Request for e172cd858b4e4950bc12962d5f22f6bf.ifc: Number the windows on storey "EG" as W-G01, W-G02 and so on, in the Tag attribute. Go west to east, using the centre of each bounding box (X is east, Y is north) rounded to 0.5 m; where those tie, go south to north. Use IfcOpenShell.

First a look at what the model holds.

```python
import ifcopenshell
import ifcopenshell.util.element
import ifcopenshell.util.placement

model = ifcopenshell.open("e172cd858b4e4950bc12962d5f22f6bf.ifc")
print(model.schema)
storey = next(s for s in model.by_type("IfcBuildingStorey") if s.Name == "EG")
windows = [e for e in ifcopenshell.util.element.get_decomposition(storey) if e.is_a("IfcWindow")]
for e in sorted(windows, key=lambda e: e.id()):
    origin = ifcopenshell.util.placement.get_local_placement(e.ObjectPlacement)[:3, 3]
    print(e.id(), e.Tag, e.Name, origin.round(2) + 0.0, sep=" | ")
```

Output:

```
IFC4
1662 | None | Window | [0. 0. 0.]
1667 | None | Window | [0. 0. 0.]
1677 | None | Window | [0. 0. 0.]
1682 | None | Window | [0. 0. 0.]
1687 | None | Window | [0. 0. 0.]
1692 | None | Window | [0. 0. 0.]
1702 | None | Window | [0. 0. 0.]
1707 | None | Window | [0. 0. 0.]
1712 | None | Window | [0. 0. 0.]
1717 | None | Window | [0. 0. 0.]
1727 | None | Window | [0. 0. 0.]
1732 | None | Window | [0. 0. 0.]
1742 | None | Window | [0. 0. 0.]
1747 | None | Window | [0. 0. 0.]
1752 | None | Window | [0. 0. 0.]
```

```python
import ifcopenshell
import ifcopenshell.geom
import ifcopenshell.util.element
import ifcopenshell.util.shape

model = ifcopenshell.open("e172cd858b4e4950bc12962d5f22f6bf.ifc")
settings = ifcopenshell.geom.settings()
settings.set("use-world-coords", True)


def centre(element):
    shape = ifcopenshell.geom.create_shape(settings, element)
    return ifcopenshell.util.shape.get_bbox_centroid(shape.geometry)


storey = next(s for s in model.by_type("IfcBuildingStorey") if s.Name == "EG")
windows = [e for e in ifcopenshell.util.element.get_decomposition(storey) if e.is_a("IfcWindow")]

# Insertion points can sit at a corner or the storey origin, so sort by the geometry (in metres).
centres = {e: centre(e) for e in windows}
windows.sort(key=lambda e: (round(centres[e][0] / 0.5), centres[e][1]))

for i, e in enumerate(windows, start=1):
    number = f"W-G{i:02d}"
    e.Tag = number
    print(e.id(), number)

model.write("e172cd858b4e4950bc12962d5f22f6bf-out.ifc")
```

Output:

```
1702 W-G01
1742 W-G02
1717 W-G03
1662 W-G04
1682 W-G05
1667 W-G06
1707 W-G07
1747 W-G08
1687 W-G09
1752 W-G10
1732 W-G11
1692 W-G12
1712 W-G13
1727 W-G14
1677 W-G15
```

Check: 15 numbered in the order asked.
